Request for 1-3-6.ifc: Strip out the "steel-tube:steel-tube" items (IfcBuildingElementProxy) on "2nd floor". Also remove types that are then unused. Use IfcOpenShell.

First a look at what the model holds.

```python
import ifcopenshell
import ifcopenshell.util.element

model = ifcopenshell.open("1-3-6.ifc")
print(model.schema)
storey = next(s for s in model.by_type("IfcBuildingStorey") if s.Name == "2nd floor")
proxies = [e for e in ifcopenshell.util.element.get_decomposition(storey) if e.is_a("IfcBuildingElementProxy")]
seen = {}
for e in proxies:
    element_type = ifcopenshell.util.element.get_type(e)
    name = element_type.Name if element_type not in (None, e) else None
    seen[name] = seen.get(name, 0) + 1
for name, count in sorted(seen.items(), key=str):
    print(count, "x", name)
```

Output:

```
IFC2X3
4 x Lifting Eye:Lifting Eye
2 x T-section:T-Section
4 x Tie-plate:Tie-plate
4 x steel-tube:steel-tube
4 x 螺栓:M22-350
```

```python
import ifcopenshell
import ifcopenshell.api.root
import ifcopenshell.util.element

model = ifcopenshell.open("1-3-6.ifc")

storey = next(s for s in model.by_type("IfcBuildingStorey") if s.Name == "2nd floor")
proxies = [e for e in ifcopenshell.util.element.get_decomposition(storey) if e.is_a("IfcBuildingElementProxy")]
targets = [e for e in proxies if (t := ifcopenshell.util.element.get_type(e)) not in (None, e) and t.Name == "steel-tube:steel-tube"]
types = {ifcopenshell.util.element.get_type(e) for e in targets} - {None, *targets}

for e in targets:
    ifcopenshell.api.root.remove_product(model, product=e)
print(len(targets), "removed")

unused = [t for t in types if not ifcopenshell.util.element.get_types(t)]
for t in unused:
    ifcopenshell.api.root.remove_product(model, product=t)
print(len(unused), "unused types removed")

model.write("1-3-6_rev.ifc")
```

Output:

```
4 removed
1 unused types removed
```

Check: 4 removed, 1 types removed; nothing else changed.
